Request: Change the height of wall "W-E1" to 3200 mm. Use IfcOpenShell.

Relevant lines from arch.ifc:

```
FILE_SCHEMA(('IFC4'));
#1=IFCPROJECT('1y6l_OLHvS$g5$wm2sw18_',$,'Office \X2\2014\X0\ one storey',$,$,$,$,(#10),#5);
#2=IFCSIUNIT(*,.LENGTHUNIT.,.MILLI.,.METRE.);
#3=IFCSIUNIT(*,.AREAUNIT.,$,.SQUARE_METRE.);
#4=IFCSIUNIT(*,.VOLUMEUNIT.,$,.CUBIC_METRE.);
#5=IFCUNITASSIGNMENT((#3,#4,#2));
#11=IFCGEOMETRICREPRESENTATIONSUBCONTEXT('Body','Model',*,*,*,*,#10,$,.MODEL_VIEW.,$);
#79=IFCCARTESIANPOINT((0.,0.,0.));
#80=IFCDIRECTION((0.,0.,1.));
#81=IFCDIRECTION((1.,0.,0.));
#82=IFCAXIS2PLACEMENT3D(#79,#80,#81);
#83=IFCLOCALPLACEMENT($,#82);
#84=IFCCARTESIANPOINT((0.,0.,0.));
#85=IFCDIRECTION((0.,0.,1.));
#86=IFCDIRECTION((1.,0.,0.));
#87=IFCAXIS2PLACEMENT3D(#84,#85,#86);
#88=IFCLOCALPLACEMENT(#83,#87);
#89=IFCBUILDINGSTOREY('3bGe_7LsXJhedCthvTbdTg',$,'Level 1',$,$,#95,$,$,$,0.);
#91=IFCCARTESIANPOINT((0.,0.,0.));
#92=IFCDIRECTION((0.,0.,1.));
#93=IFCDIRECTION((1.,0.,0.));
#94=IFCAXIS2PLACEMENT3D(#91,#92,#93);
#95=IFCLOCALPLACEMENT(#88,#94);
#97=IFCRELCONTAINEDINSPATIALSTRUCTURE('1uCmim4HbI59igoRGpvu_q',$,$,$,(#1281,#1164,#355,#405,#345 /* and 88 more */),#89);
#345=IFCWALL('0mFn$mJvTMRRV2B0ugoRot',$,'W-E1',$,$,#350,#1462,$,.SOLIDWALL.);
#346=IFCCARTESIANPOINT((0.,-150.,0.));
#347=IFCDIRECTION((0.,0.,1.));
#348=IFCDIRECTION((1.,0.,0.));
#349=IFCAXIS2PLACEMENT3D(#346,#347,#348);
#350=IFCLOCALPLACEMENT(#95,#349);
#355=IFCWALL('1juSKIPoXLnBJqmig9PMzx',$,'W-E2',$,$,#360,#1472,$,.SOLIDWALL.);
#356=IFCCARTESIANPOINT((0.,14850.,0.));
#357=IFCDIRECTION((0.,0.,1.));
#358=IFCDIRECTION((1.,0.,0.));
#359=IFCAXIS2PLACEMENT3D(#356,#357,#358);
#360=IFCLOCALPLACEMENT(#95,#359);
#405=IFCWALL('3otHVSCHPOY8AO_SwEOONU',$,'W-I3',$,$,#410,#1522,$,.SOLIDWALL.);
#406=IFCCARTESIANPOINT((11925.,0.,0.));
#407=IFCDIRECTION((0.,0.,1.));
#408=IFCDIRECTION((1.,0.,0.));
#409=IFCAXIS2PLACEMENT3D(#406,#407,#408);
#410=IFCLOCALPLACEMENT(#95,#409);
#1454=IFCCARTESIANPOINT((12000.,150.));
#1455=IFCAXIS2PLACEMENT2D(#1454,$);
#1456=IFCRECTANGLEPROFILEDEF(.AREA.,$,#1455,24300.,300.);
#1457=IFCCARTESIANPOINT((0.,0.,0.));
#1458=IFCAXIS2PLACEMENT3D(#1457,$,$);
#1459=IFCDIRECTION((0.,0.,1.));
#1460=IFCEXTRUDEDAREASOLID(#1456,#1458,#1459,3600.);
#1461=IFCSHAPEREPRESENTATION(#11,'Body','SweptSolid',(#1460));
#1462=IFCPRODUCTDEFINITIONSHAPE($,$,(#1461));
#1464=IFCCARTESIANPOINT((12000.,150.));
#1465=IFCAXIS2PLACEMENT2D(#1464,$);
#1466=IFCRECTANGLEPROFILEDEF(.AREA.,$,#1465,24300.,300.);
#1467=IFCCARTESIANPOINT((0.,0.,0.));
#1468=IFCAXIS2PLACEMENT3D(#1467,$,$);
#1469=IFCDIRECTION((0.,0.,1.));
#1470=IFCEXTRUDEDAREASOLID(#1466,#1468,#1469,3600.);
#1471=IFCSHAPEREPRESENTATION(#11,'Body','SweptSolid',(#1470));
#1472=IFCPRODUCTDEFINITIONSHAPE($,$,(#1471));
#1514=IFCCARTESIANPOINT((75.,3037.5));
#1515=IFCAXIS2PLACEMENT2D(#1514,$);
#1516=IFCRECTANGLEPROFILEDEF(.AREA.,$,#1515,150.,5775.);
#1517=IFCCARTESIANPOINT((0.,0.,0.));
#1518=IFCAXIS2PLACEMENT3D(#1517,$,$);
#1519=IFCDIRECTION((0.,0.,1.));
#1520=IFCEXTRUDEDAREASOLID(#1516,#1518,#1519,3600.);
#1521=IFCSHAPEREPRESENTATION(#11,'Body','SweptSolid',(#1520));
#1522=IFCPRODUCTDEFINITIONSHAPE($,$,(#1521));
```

```python
import ifcopenshell
import ifcopenshell.geom
import ifcopenshell.util.representation
import ifcopenshell.util.shape
import ifcopenshell.util.unit

model = ifcopenshell.open("arch.ifc")
unit_scale = ifcopenshell.util.unit.calculate_unit_scale(model)
settings = ifcopenshell.geom.settings()


def volume(element):
    """Net volume in cubic metres, openings subtracted."""
    shape = ifcopenshell.geom.create_shape(settings, element)
    return ifcopenshell.util.shape.get_volume(shape.geometry)


wall = model.by_guid("0mFn$mJvTMRRV2B0ugoRot")
before = volume(wall)

body = ifcopenshell.util.representation.get_representation(wall, "Model", "Body")
solid = body.Items[0]
old_height = solid.Depth
solid.Depth = 3.2 / unit_scale
after = volume(wall)

print(f"height {old_height:g} -> {solid.Depth:g}, volume {before:.3f} -> {after:.3f} m3")

model.write("arch_v2.ifc")
```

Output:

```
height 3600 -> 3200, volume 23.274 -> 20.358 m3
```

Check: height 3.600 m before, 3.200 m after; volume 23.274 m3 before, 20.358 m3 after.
